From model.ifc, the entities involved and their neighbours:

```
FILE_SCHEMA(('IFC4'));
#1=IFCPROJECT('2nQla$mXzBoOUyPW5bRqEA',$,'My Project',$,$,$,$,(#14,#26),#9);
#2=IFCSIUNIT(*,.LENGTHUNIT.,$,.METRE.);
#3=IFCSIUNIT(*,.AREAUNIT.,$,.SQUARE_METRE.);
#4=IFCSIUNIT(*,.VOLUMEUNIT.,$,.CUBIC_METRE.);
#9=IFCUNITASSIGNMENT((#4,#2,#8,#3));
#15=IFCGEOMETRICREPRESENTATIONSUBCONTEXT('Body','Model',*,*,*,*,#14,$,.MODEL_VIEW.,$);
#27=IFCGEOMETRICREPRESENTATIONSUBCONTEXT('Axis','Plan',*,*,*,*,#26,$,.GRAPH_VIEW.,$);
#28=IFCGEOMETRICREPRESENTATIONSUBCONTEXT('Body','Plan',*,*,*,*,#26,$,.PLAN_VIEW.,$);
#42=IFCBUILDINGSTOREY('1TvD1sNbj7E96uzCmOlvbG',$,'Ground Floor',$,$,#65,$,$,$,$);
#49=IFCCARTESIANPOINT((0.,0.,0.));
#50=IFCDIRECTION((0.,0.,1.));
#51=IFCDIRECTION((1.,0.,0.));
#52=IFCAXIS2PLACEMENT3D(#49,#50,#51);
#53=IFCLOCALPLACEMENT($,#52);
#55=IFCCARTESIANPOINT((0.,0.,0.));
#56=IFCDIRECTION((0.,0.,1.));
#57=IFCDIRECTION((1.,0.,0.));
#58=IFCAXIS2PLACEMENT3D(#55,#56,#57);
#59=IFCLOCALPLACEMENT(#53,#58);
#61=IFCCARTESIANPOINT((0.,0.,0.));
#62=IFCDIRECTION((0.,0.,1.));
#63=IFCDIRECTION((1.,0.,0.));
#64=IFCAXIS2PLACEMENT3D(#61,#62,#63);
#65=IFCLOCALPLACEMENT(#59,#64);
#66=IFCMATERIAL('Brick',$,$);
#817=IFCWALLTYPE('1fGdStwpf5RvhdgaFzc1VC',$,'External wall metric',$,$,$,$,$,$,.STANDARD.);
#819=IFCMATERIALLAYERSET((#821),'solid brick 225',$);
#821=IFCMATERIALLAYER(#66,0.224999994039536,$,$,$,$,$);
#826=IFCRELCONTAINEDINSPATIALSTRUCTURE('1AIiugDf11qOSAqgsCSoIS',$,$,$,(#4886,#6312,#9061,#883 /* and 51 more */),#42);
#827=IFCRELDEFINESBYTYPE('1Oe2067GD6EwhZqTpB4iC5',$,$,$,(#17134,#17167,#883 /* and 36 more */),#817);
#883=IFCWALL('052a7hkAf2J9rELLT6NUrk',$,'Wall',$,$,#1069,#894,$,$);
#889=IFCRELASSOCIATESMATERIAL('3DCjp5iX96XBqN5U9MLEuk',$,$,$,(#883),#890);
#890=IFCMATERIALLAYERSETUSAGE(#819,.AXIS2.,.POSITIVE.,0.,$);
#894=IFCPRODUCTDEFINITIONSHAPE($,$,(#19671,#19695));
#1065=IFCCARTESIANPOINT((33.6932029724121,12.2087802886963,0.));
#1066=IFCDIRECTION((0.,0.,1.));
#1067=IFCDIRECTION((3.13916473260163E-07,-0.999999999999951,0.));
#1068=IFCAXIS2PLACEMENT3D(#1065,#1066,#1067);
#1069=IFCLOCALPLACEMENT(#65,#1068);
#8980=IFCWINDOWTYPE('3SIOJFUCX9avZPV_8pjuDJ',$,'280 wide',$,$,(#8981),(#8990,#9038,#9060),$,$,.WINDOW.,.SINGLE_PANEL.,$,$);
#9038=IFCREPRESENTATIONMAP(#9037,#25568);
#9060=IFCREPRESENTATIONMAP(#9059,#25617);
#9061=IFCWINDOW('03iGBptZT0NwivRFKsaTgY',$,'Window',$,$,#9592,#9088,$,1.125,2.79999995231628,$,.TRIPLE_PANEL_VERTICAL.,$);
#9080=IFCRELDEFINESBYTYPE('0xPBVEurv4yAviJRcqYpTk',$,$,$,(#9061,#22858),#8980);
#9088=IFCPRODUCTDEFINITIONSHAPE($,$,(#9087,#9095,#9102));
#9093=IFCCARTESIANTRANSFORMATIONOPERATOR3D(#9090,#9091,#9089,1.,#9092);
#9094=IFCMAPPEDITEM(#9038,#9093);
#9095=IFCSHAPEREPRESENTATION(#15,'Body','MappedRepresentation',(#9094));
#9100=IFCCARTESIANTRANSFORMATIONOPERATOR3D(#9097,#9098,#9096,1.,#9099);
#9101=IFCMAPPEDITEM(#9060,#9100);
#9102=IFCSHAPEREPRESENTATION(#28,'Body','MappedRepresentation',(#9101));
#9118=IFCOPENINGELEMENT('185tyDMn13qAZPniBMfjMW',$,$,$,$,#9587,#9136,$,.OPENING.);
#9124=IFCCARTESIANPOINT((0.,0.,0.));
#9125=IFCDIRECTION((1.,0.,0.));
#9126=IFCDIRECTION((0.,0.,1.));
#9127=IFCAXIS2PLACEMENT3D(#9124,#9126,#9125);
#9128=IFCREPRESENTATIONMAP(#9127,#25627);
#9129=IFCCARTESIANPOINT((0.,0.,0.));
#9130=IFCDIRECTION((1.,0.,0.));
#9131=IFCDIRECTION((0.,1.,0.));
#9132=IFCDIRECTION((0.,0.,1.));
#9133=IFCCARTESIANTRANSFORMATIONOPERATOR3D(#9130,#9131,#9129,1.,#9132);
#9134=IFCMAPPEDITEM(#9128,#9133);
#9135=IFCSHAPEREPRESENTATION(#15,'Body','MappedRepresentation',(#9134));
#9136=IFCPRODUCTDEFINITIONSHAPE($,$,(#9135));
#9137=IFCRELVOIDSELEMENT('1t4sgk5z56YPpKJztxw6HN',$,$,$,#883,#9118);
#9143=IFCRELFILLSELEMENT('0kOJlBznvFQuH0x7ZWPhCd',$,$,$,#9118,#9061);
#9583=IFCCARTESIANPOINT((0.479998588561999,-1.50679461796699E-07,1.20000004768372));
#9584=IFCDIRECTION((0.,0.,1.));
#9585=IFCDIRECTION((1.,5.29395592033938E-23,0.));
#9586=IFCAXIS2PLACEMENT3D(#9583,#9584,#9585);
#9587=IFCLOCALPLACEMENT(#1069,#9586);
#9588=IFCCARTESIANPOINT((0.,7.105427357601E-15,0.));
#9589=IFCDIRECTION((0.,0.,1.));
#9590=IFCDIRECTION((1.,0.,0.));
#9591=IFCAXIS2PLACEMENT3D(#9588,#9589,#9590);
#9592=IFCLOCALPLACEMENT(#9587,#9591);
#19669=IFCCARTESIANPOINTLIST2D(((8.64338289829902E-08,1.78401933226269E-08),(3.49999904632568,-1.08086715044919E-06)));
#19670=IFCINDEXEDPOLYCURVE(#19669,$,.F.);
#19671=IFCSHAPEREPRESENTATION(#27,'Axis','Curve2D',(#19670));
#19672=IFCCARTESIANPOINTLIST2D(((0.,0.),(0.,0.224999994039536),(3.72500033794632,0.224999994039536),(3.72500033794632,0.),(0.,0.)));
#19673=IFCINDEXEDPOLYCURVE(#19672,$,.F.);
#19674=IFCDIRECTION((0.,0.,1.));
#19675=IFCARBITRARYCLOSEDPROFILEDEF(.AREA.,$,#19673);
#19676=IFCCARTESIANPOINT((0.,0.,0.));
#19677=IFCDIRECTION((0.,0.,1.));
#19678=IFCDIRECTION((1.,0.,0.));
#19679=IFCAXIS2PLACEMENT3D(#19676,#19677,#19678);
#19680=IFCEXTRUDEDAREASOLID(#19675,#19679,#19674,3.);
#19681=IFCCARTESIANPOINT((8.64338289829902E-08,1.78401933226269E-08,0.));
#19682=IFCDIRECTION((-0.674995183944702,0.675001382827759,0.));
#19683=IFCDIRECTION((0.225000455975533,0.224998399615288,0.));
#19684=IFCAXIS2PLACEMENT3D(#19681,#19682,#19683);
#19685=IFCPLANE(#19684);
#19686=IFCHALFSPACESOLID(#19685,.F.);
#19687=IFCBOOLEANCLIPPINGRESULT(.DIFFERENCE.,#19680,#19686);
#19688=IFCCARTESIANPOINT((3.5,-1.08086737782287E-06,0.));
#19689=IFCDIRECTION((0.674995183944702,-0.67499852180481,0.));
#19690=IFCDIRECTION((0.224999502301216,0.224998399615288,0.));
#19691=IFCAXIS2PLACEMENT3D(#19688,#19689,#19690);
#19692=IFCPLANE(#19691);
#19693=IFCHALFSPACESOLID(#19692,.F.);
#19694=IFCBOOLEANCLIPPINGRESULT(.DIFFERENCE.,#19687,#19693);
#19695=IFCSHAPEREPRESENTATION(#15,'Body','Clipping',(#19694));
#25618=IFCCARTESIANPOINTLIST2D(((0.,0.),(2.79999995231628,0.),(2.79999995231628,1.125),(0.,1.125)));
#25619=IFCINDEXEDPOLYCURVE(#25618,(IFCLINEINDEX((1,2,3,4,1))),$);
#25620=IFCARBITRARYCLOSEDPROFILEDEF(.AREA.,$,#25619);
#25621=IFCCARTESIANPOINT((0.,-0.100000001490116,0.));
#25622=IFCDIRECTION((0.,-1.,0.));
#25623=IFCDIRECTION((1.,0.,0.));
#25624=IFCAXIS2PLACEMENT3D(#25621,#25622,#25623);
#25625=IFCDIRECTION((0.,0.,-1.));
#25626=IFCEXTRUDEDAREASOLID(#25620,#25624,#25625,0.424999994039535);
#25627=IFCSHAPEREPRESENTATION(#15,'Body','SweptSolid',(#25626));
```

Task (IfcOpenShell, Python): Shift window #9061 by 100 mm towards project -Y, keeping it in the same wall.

```python
import ifcopenshell
import ifcopenshell.api.geometry
import ifcopenshell.util.placement
import ifcopenshell.util.unit

model = ifcopenshell.open("model.ifc")
unit_scale = ifcopenshell.util.unit.calculate_unit_scale(model)

window = model.by_id(9061)
opening = window.FillsVoids[0].RelatingOpeningElement
wall = opening.VoidsElements[0].RelatingBuildingElement

wall_matrix = ifcopenshell.util.placement.get_local_placement(wall.ObjectPlacement)
shift = wall_matrix[:3, 0] * 0.1 / unit_scale
before = ifcopenshell.util.placement.get_local_placement(window.ObjectPlacement)[:3, 3].copy()

# The window is placed relative to its opening, so it follows when the opening moves.
matrix = ifcopenshell.util.placement.get_local_placement(opening.ObjectPlacement)
matrix[:3, 3] += shift
ifcopenshell.api.geometry.edit_object_placement(
    model, product=opening, matrix=matrix, is_si=False, should_transform_children=True
)

after = ifcopenshell.util.placement.get_local_placement(window.ObjectPlacement)[:3, 3]
print("window moved by", (after - before).round(3) + 0.0)

model.write("model_rev.ifc")
```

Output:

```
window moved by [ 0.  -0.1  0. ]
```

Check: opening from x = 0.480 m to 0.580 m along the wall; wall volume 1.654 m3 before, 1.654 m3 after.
